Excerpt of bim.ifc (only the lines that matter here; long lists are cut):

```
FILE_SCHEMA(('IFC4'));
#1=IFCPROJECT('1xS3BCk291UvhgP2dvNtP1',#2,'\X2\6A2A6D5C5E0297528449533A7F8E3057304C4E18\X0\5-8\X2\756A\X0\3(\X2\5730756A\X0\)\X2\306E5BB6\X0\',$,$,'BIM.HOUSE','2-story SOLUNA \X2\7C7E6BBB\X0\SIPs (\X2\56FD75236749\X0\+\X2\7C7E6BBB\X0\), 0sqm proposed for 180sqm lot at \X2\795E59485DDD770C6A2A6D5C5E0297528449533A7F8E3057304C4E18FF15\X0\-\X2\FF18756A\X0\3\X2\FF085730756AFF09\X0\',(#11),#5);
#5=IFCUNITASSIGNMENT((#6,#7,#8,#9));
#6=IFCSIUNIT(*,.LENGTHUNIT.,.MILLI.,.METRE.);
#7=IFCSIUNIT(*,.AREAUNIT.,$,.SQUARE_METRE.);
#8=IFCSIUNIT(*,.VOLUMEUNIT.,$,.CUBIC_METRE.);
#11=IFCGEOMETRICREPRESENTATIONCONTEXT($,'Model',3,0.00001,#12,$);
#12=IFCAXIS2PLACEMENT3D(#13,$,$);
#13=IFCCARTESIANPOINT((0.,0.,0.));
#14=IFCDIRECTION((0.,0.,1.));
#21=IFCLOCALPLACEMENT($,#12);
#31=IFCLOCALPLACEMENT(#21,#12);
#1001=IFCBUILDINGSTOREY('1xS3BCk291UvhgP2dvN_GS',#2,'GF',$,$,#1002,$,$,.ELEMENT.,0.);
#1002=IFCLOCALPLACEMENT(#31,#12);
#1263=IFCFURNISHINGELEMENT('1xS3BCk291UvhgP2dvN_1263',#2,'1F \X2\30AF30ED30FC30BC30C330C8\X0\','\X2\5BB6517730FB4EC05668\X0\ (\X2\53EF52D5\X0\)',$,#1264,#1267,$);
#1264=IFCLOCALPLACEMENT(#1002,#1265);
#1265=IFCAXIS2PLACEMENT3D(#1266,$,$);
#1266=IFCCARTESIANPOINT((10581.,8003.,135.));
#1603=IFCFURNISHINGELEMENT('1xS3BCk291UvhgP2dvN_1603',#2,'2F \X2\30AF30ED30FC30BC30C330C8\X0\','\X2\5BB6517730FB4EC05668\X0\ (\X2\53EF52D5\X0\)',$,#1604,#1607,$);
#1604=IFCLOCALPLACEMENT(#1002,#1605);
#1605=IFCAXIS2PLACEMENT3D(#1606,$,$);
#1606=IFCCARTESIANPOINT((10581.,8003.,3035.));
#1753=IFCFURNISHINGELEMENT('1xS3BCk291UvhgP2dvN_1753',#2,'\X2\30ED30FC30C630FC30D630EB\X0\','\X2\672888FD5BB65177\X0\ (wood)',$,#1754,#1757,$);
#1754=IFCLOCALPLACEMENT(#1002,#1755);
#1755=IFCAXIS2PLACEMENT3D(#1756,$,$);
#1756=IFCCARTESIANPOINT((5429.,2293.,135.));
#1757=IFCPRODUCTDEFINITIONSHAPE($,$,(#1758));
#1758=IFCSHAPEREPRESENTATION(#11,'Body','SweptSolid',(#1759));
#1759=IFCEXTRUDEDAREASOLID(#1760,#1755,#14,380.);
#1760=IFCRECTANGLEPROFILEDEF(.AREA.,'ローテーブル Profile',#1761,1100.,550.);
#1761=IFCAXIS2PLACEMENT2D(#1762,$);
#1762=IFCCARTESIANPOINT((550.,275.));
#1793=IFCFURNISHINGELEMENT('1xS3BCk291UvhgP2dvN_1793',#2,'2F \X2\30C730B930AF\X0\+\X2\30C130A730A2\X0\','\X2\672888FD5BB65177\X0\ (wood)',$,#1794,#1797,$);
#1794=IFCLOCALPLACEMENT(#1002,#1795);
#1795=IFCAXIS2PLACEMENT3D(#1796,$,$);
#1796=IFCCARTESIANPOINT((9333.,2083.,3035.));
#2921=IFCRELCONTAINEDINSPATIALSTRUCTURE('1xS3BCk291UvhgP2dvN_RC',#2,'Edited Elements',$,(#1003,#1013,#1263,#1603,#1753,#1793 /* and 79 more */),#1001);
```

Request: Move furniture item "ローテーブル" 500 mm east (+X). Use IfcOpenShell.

```python
import ifcopenshell
import ifcopenshell.api.geometry
import ifcopenshell.util.placement
import ifcopenshell.util.unit

model = ifcopenshell.open("bim.ifc")
unit_scale = ifcopenshell.util.unit.calculate_unit_scale(model)

item = model.by_guid("1xS3BCk291UvhgP2dvN_1753")
matrix = ifcopenshell.util.placement.get_local_placement(item.ObjectPlacement)
matrix[0, 3] += 0.5 / unit_scale
ifcopenshell.api.geometry.edit_object_placement(model, product=item, matrix=matrix, is_si=False)

print(ifcopenshell.util.placement.get_local_placement(item.ObjectPlacement).round(3) + 0.0)

model.write("bim-out.ifc")
```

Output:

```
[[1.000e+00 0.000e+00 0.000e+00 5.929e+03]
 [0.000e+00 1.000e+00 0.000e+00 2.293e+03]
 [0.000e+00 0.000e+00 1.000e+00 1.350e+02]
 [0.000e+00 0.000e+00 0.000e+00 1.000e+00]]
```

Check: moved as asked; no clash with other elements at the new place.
